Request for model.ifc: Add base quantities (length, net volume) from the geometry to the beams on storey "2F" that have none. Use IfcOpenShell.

First a look at what the model holds.

```python
import ifcopenshell
import ifcopenshell.util.element
import ifcopenshell.util.unit

model = ifcopenshell.open("model.ifc")
print(model.schema)
for unit_type in ("LENGTHUNIT", "AREAUNIT", "VOLUMEUNIT"):
    print(unit_type, ifcopenshell.util.unit.calculate_unit_scale(model, unit_type))
storey = next(s for s in model.by_type("IfcBuildingStorey") if s.Name == "2F")
beams = [e for e in ifcopenshell.util.element.get_decomposition(storey) if e.is_a("IfcBeam")]
for e in sorted(beams, key=lambda e: e.id()):
    print(e.id(), e.is_a(), e.Name, list(ifcopenshell.util.element.get_psets(e, qtos_only=True)), sep=" | ")
```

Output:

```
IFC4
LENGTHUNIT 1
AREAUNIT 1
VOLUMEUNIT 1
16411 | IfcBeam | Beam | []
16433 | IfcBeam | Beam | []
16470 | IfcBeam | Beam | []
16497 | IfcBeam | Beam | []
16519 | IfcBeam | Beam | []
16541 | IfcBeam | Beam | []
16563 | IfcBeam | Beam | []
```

```python
import ifcopenshell
import ifcopenshell.api.pset
import ifcopenshell.geom
import ifcopenshell.util.element
import ifcopenshell.util.shape
import ifcopenshell.util.unit

model = ifcopenshell.open("model.ifc")
unit_scale = ifcopenshell.util.unit.calculate_unit_scale(model)
volume_scale = ifcopenshell.util.unit.calculate_unit_scale(model, "VOLUMEUNIT")
settings = ifcopenshell.geom.settings()

storey = next(s for s in model.by_type("IfcBuildingStorey") if s.Name == "2F")
beams = [e for e in ifcopenshell.util.element.get_decomposition(storey) if e.is_a("IfcBeam")]

for e in sorted(beams, key=lambda e: e.id()):
    if ifcopenshell.util.element.get_psets(e, qtos_only=True, should_inherit=False):
        continue
    # Geometry comes back in metres, in the element's own axes.
    shape = ifcopenshell.geom.create_shape(settings, e)
    values = {
        "Length": ifcopenshell.util.shape.get_max_xyz(shape.geometry) / unit_scale,
        "NetVolume": ifcopenshell.util.shape.get_volume(shape.geometry) / volume_scale,
    }
    qto = ifcopenshell.api.pset.add_qto(model, product=e, name="Qto_BeamBaseQuantities")
    ifcopenshell.api.pset.edit_qto(model, qto=qto, properties=values)
    print(e.id(), {k: round(v, 3) for k, v in values.items()})

model.write("model_edited.ifc")
```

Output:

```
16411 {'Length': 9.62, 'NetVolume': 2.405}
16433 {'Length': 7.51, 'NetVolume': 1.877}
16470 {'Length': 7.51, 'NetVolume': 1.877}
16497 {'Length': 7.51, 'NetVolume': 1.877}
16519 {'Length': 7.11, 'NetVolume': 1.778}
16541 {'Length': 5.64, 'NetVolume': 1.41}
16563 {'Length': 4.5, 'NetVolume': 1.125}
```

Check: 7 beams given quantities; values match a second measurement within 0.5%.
